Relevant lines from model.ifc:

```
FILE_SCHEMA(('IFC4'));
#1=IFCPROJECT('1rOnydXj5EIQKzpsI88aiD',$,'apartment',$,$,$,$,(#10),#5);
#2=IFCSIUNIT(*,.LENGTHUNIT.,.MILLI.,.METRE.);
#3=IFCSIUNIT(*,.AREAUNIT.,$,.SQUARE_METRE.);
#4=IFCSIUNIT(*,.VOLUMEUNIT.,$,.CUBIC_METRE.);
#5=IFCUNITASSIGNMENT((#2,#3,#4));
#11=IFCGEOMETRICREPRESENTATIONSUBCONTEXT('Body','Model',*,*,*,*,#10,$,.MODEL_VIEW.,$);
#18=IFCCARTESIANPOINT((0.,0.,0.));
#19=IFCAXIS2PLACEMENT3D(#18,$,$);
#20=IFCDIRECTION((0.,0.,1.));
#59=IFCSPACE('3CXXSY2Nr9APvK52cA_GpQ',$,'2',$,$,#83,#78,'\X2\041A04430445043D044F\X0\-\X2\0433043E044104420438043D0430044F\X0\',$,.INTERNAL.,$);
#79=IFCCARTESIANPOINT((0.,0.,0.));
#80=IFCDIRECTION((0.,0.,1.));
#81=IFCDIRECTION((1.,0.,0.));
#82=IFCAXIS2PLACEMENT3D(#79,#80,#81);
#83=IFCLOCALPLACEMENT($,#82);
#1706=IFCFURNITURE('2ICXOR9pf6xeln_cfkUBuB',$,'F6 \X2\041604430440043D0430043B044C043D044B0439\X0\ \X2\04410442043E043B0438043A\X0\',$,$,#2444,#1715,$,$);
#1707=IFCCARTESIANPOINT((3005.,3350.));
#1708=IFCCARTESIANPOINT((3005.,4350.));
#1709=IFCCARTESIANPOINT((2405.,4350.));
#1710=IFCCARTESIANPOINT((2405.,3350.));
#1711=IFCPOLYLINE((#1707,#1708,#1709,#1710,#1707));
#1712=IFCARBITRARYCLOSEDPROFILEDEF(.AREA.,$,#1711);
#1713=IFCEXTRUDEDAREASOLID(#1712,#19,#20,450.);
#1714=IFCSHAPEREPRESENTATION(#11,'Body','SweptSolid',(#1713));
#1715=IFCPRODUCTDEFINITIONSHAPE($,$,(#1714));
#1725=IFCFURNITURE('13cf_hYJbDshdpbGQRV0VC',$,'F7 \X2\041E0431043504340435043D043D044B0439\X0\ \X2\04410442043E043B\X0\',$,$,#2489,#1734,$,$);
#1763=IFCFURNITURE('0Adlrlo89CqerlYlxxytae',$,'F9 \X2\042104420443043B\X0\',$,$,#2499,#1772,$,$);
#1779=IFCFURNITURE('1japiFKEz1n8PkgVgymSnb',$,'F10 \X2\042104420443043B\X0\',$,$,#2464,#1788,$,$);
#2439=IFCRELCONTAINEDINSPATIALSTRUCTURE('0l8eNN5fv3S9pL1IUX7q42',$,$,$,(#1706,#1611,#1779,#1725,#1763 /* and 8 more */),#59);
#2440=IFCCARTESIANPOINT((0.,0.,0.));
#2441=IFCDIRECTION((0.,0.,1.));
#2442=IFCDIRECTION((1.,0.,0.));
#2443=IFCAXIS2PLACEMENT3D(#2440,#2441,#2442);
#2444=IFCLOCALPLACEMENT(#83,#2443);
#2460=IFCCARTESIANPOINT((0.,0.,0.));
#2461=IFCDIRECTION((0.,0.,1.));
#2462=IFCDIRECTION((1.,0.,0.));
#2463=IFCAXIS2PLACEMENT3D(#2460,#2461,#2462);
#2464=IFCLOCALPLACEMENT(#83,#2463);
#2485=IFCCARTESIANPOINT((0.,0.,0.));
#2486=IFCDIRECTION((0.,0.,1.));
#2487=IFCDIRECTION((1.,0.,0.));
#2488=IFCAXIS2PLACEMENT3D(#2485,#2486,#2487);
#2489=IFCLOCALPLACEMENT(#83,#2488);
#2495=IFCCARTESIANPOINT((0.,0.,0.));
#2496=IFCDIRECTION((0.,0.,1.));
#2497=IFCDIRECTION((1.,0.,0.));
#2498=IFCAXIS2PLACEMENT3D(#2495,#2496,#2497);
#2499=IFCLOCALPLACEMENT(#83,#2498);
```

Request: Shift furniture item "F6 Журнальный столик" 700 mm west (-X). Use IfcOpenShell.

```python
import ifcopenshell
import ifcopenshell.api.geometry
import ifcopenshell.util.placement
import ifcopenshell.util.unit

model = ifcopenshell.open("model.ifc")
unit_scale = ifcopenshell.util.unit.calculate_unit_scale(model)

item = model.by_guid("2ICXOR9pf6xeln_cfkUBuB")
matrix = ifcopenshell.util.placement.get_local_placement(item.ObjectPlacement)
matrix[0, 3] -= 0.7 / unit_scale
ifcopenshell.api.geometry.edit_object_placement(model, product=item, matrix=matrix, is_si=False)

print(ifcopenshell.util.placement.get_local_placement(item.ObjectPlacement).round(3) + 0.0)

model.write("model-out.ifc")
```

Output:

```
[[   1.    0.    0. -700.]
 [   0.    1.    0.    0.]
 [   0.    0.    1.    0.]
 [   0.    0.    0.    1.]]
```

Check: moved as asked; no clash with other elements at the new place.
